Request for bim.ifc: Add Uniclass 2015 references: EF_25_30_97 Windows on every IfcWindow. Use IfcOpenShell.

First a look at what the model holds.

```python
import ifcopenshell

model = ifcopenshell.open("bim.ifc")
print(model.schema)
print("classifications:", [c.Name for c in model.by_type("IfcClassification")])
for ifc_class in ("IfcDoor", "IfcRoof", "IfcStair", "IfcWall", "IfcWindow"):
    print(ifc_class, len(model.by_type(ifc_class)))
```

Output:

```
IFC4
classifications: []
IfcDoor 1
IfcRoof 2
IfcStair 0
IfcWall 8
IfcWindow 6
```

```python
import ifcopenshell
import ifcopenshell.api.classification

model = ifcopenshell.open("bim.ifc")

system = ifcopenshell.api.classification.add_classification(model, classification="Uniclass 2015")

codes = {
    "IfcWindow": ("EF_25_30_97", "Windows"),
}
for ifc_class, (code, name) in codes.items():
    products = model.by_type(ifc_class)
    ifcopenshell.api.classification.add_reference(
        model, products=products, classification=system, identification=code, name=name
    )
    print(code, len(products))

model.write("bim_v2.ifc")
```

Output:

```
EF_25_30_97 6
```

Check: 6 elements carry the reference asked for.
